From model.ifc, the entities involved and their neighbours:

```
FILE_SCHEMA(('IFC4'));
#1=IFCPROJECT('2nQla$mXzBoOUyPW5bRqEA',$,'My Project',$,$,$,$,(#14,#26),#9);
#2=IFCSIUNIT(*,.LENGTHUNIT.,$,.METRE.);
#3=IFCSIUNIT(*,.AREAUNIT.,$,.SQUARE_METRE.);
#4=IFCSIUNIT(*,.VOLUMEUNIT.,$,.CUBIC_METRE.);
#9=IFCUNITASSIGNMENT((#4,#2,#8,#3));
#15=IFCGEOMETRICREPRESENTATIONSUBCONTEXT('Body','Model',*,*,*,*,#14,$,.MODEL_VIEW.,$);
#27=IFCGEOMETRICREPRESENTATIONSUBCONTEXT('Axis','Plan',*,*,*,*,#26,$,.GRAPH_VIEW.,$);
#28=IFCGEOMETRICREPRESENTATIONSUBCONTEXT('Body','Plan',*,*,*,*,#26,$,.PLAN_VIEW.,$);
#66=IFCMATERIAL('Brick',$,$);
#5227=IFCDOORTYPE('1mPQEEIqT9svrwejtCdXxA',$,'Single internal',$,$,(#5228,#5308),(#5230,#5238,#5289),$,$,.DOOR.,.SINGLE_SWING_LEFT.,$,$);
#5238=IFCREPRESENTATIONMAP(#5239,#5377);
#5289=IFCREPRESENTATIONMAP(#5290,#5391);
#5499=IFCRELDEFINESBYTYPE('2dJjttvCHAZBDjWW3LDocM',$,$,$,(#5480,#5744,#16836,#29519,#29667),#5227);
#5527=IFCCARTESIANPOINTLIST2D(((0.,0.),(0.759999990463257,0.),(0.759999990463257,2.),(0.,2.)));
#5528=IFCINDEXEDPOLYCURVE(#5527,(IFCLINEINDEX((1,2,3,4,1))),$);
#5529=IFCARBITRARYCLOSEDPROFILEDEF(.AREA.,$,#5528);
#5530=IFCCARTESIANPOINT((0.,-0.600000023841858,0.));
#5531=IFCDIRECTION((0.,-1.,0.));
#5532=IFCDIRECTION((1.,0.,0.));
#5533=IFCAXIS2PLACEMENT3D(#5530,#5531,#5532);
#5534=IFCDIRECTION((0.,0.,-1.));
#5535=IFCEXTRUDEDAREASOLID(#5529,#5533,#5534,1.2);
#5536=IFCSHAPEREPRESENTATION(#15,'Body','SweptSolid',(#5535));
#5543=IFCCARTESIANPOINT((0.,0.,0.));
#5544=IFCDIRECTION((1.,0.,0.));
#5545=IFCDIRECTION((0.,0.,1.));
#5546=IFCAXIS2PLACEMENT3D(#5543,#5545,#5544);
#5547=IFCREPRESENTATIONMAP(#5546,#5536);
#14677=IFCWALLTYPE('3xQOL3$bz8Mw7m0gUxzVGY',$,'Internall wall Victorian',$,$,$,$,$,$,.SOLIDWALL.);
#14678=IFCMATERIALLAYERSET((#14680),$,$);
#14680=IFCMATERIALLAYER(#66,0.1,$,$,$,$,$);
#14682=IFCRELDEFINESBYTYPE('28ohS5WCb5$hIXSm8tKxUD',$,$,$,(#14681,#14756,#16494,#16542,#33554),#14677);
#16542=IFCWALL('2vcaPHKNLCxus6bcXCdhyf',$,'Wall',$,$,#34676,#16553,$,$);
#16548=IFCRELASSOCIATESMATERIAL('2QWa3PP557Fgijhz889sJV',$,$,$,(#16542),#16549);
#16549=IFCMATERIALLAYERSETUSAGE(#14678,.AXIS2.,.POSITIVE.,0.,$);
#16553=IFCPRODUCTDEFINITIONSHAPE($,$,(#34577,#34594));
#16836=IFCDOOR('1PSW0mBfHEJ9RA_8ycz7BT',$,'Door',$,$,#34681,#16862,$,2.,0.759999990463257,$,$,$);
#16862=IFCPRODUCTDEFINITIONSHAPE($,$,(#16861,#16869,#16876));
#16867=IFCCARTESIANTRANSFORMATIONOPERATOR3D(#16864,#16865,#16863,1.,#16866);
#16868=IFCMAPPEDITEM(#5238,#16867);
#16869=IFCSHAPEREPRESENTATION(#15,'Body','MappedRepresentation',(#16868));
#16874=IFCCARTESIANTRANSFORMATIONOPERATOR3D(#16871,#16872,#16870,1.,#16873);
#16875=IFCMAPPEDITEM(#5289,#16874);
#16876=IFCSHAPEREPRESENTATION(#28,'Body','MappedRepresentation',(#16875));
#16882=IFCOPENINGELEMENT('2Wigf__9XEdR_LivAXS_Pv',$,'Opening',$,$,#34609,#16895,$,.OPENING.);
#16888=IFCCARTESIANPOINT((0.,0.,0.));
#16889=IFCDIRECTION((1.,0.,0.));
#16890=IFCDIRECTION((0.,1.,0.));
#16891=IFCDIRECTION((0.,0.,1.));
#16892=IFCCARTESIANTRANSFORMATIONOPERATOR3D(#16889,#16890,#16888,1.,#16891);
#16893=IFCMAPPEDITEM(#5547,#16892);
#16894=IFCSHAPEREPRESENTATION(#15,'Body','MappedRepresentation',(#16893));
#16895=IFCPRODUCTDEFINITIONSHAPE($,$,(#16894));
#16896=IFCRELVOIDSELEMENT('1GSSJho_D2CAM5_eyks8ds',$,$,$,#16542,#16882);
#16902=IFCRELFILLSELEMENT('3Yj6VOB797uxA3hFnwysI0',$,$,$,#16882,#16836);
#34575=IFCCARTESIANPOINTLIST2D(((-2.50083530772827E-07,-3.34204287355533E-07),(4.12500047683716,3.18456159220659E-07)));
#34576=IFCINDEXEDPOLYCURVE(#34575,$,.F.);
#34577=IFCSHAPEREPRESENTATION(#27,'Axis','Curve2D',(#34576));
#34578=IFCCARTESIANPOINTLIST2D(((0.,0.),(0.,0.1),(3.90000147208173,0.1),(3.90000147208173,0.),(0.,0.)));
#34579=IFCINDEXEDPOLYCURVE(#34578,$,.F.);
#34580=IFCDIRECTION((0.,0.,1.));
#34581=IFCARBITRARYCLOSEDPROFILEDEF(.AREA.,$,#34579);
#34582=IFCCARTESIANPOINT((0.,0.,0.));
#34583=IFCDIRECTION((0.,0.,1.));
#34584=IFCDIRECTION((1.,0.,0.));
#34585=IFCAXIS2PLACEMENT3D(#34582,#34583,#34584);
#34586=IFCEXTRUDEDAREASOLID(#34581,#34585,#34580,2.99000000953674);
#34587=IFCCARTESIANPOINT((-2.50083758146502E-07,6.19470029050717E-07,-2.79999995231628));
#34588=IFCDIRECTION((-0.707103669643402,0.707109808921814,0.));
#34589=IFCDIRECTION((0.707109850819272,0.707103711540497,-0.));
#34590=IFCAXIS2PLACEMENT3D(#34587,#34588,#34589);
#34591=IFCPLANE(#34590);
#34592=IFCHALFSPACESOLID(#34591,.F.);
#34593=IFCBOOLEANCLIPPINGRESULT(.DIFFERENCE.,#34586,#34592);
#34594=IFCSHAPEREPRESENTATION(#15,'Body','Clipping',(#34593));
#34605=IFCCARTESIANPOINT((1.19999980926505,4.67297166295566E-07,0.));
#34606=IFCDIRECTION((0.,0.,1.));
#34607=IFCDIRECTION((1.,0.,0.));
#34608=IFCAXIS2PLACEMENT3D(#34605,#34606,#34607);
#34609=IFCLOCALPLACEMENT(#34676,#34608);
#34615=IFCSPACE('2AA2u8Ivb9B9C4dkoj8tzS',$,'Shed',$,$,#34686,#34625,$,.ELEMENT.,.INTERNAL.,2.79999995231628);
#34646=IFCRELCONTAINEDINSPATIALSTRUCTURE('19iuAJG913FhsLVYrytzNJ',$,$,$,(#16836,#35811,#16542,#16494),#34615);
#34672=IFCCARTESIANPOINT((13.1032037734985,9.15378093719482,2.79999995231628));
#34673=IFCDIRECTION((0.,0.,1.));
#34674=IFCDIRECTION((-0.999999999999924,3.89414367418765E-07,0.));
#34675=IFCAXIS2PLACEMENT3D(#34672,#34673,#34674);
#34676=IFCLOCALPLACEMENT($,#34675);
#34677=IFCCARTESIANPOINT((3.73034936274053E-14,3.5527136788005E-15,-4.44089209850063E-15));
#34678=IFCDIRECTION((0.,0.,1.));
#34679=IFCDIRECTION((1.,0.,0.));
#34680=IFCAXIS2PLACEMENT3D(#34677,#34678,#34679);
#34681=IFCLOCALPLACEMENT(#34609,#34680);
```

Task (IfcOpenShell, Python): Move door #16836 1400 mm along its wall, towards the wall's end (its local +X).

```python
import ifcopenshell
import ifcopenshell.api.geometry
import ifcopenshell.util.placement
import ifcopenshell.util.unit

model = ifcopenshell.open("model.ifc")
unit_scale = ifcopenshell.util.unit.calculate_unit_scale(model)

door = model.by_guid("1PSW0mBfHEJ9RA_8ycz7BT")
opening = door.FillsVoids[0].RelatingOpeningElement
wall = opening.VoidsElements[0].RelatingBuildingElement

wall_matrix = ifcopenshell.util.placement.get_local_placement(wall.ObjectPlacement)
shift = wall_matrix[:3, 0] * 1.4 / unit_scale
before = ifcopenshell.util.placement.get_local_placement(door.ObjectPlacement)[:3, 3].copy()

# The door is placed relative to its opening, so it follows when the opening moves.
matrix = ifcopenshell.util.placement.get_local_placement(opening.ObjectPlacement)
matrix[:3, 3] += shift
ifcopenshell.api.geometry.edit_object_placement(
    model, product=opening, matrix=matrix, is_si=False, should_transform_children=True
)

after = ifcopenshell.util.placement.get_local_placement(door.ObjectPlacement)[:3, 3]
print("door moved by", (after - before).round(3) + 0.0)

model.write("model-out.ifc")
```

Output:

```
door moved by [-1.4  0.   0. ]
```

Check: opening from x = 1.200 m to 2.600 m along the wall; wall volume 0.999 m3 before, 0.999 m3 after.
